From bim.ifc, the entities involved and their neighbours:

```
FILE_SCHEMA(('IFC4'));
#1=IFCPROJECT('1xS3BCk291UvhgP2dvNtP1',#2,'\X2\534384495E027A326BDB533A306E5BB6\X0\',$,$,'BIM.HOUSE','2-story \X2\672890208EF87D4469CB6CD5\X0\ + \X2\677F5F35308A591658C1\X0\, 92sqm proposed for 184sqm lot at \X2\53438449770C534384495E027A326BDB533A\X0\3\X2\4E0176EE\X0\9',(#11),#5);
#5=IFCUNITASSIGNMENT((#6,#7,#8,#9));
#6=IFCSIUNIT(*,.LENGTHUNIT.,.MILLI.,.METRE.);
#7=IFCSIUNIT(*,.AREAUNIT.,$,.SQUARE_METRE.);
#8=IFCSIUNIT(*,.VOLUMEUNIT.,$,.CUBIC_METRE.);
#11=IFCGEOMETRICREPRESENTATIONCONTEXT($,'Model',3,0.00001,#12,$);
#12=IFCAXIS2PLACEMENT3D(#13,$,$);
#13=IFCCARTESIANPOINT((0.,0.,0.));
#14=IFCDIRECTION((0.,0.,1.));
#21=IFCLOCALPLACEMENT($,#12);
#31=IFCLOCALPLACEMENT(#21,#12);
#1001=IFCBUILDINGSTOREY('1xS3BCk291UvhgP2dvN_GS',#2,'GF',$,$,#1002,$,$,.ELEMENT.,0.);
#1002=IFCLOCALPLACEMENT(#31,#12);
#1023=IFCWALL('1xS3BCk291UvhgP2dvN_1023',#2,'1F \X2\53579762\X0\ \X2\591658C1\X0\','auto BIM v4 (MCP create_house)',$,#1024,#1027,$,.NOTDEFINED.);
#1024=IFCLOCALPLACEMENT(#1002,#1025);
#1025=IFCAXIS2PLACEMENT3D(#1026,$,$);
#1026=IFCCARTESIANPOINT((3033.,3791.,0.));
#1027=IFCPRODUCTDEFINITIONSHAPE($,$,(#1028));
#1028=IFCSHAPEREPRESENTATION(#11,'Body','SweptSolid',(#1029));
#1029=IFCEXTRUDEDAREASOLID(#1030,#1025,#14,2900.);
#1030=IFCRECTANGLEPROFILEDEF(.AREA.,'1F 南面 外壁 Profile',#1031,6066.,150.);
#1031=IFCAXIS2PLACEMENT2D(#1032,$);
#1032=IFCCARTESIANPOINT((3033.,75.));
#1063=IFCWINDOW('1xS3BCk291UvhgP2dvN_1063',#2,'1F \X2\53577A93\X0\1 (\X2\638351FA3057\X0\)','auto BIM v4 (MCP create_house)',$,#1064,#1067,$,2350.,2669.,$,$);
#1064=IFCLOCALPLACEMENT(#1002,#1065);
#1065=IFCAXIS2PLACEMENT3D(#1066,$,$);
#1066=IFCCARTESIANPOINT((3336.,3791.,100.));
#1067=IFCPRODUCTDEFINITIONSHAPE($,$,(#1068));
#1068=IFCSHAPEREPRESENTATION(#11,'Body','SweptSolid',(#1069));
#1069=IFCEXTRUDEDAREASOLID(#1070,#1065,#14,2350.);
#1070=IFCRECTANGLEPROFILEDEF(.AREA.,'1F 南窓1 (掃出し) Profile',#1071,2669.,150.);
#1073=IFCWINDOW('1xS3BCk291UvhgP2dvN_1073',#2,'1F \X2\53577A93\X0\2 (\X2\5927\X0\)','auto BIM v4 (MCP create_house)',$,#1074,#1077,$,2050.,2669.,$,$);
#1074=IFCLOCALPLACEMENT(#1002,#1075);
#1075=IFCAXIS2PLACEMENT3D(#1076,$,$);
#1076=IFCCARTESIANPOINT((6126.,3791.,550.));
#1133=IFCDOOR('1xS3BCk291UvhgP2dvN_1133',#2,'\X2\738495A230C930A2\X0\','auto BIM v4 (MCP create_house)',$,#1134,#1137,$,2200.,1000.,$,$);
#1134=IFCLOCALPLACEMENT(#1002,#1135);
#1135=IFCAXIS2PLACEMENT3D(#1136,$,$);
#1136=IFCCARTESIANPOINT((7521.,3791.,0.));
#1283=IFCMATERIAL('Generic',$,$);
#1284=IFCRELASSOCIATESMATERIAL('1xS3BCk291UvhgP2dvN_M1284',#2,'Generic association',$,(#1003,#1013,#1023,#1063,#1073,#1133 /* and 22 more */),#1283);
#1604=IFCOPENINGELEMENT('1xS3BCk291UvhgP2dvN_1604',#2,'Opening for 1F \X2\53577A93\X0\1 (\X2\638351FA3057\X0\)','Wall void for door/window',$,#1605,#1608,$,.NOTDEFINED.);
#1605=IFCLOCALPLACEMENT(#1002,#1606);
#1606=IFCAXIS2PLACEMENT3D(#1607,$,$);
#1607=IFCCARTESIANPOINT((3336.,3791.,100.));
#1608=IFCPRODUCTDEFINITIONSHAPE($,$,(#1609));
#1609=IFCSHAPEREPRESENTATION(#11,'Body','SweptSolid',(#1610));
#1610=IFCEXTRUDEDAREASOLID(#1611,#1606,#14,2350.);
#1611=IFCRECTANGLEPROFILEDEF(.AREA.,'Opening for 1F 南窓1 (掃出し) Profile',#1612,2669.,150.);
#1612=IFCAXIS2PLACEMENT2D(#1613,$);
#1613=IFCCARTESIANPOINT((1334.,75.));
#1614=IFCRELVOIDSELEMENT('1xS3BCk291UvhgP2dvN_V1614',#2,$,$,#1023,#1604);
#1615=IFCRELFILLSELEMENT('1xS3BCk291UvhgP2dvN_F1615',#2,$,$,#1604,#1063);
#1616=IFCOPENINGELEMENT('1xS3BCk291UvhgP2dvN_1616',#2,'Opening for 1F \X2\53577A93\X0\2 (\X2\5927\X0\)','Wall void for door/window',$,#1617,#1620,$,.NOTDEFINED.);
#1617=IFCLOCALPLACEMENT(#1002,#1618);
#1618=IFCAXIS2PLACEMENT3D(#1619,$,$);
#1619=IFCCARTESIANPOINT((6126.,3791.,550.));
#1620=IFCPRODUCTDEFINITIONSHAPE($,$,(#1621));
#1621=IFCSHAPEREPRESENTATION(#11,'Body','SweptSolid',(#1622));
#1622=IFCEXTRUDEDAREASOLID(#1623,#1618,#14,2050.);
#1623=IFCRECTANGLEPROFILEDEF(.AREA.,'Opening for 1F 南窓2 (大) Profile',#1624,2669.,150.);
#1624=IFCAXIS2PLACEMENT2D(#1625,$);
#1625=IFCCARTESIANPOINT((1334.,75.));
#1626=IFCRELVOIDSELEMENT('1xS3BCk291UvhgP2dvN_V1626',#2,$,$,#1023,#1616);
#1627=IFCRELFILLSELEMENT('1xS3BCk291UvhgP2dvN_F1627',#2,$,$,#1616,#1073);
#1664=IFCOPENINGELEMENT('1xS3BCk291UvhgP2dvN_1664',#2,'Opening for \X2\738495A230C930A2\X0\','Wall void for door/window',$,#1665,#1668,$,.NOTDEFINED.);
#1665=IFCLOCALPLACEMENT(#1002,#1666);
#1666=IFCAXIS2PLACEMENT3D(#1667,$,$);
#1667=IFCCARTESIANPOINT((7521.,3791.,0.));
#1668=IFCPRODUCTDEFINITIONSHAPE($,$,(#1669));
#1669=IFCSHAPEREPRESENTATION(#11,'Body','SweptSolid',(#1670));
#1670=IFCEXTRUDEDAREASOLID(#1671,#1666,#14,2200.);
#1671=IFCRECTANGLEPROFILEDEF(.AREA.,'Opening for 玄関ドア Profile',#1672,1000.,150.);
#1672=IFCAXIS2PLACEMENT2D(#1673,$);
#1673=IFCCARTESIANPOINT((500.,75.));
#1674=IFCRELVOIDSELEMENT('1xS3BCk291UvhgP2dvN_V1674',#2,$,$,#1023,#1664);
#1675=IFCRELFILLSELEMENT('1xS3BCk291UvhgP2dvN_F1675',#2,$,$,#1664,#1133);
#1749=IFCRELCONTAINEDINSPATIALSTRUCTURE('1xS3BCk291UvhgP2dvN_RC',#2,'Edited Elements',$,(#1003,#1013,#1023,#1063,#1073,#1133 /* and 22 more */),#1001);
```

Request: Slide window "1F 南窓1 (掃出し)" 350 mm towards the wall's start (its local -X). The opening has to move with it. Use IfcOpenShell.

```python
import ifcopenshell
import ifcopenshell.api.geometry
import ifcopenshell.util.placement
import ifcopenshell.util.unit

model = ifcopenshell.open("bim.ifc")
unit_scale = ifcopenshell.util.unit.calculate_unit_scale(model)

window = model.by_guid("1xS3BCk291UvhgP2dvN_1063")
opening = window.FillsVoids[0].RelatingOpeningElement
wall = opening.VoidsElements[0].RelatingBuildingElement

wall_matrix = ifcopenshell.util.placement.get_local_placement(wall.ObjectPlacement)
shift = wall_matrix[:3, 0] * -0.35 / unit_scale
before = ifcopenshell.util.placement.get_local_placement(window.ObjectPlacement)[:3, 3].copy()

# The window is not placed relative to its opening, so move both.
for product in (opening, window):
    matrix = ifcopenshell.util.placement.get_local_placement(product.ObjectPlacement)
    matrix[:3, 3] += shift
    ifcopenshell.api.geometry.edit_object_placement(model, product=product, matrix=matrix, is_si=False)

after = ifcopenshell.util.placement.get_local_placement(window.ObjectPlacement)[:3, 3]
print("window moved by", (after - before).round(3) + 0.0)

model.write("bim_rev.ifc")
```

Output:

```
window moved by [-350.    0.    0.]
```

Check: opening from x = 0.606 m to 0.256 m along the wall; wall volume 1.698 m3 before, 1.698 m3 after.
